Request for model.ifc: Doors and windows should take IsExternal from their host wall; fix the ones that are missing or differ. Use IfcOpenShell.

First a look at what the model holds.

```python
import ifcopenshell
import ifcopenshell.util.element

model = ifcopenshell.open("model.ifc")
print(model.schema)
seen = {}
for e in model.by_type("IfcDoor") + model.by_type("IfcWindow"):
    if not e.FillsVoids:
        continue
    host = e.FillsVoids[0].RelatingOpeningElement.VoidsElements[0].RelatingBuildingElement
    own = ifcopenshell.util.element.get_pset(e, f"Pset_{e.is_a()[3:].removesuffix('StandardCase')}Common", "IsExternal")
    wall = ifcopenshell.util.element.get_pset(host, "Pset_WallCommon", "IsExternal")
    seen[e.is_a(), own, wall] = seen.get((e.is_a(), own, wall), 0) + 1
for (cls, own, wall), count in sorted(seen.items(), key=str):
    print(count, cls, "IsExternal:", own, "| host wall:", wall)
```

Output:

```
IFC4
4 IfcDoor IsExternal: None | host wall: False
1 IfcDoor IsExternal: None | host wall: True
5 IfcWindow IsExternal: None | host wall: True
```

```python
import ifcopenshell
import ifcopenshell.api.pset
import ifcopenshell.util.element

model = ifcopenshell.open("model.ifc")

count = 0
for ifc_class, pset_name in (("IfcDoor", "Pset_DoorCommon"), ("IfcWindow", "Pset_WindowCommon")):
    for e in model.by_type(ifc_class):
        if not e.FillsVoids:
            continue
        host = e.FillsVoids[0].RelatingOpeningElement.VoidsElements[0].RelatingBuildingElement
        external = ifcopenshell.util.element.get_pset(host, "Pset_WallCommon", "IsExternal")
        if external is None or ifcopenshell.util.element.get_pset(e, pset_name, "IsExternal") == external:
            continue
        pset = ifcopenshell.api.pset.add_pset(model, product=e, name=pset_name)
        ifcopenshell.api.pset.edit_pset(model, pset=pset, properties={"IsExternal": external})
        count += 1

print(count, "updated")

model.write("model_v2.ifc")
```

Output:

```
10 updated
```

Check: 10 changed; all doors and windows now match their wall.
